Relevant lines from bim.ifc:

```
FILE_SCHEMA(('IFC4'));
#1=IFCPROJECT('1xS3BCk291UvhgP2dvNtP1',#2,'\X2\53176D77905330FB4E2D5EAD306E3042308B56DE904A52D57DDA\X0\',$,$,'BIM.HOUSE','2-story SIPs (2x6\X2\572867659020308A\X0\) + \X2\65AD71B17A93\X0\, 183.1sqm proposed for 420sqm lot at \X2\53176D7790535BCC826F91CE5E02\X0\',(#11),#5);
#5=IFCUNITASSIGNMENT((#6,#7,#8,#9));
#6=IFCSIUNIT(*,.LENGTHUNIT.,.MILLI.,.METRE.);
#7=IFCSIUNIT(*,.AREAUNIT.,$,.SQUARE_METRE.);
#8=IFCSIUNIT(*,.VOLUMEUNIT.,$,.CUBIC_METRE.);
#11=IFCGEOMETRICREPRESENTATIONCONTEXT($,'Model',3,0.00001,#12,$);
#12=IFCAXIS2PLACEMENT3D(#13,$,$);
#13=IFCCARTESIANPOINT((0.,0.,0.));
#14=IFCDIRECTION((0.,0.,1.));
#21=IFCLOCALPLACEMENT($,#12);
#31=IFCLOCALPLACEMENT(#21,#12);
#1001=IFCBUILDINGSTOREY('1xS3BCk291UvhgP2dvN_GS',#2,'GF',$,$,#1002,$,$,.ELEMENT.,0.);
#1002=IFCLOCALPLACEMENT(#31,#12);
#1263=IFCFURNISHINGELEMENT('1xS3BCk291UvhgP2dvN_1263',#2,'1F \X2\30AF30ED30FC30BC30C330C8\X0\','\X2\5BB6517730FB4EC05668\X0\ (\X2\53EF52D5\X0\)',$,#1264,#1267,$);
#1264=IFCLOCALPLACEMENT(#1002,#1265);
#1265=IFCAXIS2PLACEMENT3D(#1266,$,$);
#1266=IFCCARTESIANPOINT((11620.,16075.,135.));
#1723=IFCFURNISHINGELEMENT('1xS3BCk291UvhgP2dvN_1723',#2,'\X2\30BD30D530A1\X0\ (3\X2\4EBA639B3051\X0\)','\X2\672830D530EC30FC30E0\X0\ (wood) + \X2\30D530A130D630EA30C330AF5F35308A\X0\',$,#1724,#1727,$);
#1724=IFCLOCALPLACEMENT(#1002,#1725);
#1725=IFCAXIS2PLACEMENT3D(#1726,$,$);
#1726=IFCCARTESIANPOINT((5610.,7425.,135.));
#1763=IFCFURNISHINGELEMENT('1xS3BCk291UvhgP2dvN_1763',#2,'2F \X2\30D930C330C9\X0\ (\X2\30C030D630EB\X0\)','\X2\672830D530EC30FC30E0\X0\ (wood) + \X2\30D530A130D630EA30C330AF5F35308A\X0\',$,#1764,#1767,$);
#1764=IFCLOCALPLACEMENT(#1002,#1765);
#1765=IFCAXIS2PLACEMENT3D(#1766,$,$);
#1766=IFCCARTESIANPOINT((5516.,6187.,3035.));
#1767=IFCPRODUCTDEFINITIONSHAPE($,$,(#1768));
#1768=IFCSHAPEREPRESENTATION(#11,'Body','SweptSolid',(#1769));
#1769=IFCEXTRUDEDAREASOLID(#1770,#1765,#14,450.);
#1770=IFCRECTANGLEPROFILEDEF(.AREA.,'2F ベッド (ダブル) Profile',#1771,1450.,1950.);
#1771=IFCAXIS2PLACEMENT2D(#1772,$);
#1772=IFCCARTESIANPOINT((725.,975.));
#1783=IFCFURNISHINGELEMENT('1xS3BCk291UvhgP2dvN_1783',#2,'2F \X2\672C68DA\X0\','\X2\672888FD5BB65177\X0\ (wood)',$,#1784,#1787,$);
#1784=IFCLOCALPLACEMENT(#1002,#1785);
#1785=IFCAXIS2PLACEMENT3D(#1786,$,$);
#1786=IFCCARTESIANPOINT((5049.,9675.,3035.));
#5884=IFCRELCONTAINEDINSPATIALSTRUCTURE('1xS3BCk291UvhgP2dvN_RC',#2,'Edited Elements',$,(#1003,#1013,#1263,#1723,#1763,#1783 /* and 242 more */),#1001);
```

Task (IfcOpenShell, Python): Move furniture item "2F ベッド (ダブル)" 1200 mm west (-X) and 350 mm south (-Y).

```python
import ifcopenshell
import ifcopenshell.api.geometry
import ifcopenshell.util.placement
import ifcopenshell.util.unit

model = ifcopenshell.open("bim.ifc")
unit_scale = ifcopenshell.util.unit.calculate_unit_scale(model)

item = model.by_guid("1xS3BCk291UvhgP2dvN_1763")
matrix = ifcopenshell.util.placement.get_local_placement(item.ObjectPlacement)
matrix[0, 3] -= 1.2 / unit_scale
matrix[1, 3] -= 0.35 / unit_scale
ifcopenshell.api.geometry.edit_object_placement(model, product=item, matrix=matrix, is_si=False)

print(ifcopenshell.util.placement.get_local_placement(item.ObjectPlacement).round(3) + 0.0)

model.write("bim-out.ifc")
```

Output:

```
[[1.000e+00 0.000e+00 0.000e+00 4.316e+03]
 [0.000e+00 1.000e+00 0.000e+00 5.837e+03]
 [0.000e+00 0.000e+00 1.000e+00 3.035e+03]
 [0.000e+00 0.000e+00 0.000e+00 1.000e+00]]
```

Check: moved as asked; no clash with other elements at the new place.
